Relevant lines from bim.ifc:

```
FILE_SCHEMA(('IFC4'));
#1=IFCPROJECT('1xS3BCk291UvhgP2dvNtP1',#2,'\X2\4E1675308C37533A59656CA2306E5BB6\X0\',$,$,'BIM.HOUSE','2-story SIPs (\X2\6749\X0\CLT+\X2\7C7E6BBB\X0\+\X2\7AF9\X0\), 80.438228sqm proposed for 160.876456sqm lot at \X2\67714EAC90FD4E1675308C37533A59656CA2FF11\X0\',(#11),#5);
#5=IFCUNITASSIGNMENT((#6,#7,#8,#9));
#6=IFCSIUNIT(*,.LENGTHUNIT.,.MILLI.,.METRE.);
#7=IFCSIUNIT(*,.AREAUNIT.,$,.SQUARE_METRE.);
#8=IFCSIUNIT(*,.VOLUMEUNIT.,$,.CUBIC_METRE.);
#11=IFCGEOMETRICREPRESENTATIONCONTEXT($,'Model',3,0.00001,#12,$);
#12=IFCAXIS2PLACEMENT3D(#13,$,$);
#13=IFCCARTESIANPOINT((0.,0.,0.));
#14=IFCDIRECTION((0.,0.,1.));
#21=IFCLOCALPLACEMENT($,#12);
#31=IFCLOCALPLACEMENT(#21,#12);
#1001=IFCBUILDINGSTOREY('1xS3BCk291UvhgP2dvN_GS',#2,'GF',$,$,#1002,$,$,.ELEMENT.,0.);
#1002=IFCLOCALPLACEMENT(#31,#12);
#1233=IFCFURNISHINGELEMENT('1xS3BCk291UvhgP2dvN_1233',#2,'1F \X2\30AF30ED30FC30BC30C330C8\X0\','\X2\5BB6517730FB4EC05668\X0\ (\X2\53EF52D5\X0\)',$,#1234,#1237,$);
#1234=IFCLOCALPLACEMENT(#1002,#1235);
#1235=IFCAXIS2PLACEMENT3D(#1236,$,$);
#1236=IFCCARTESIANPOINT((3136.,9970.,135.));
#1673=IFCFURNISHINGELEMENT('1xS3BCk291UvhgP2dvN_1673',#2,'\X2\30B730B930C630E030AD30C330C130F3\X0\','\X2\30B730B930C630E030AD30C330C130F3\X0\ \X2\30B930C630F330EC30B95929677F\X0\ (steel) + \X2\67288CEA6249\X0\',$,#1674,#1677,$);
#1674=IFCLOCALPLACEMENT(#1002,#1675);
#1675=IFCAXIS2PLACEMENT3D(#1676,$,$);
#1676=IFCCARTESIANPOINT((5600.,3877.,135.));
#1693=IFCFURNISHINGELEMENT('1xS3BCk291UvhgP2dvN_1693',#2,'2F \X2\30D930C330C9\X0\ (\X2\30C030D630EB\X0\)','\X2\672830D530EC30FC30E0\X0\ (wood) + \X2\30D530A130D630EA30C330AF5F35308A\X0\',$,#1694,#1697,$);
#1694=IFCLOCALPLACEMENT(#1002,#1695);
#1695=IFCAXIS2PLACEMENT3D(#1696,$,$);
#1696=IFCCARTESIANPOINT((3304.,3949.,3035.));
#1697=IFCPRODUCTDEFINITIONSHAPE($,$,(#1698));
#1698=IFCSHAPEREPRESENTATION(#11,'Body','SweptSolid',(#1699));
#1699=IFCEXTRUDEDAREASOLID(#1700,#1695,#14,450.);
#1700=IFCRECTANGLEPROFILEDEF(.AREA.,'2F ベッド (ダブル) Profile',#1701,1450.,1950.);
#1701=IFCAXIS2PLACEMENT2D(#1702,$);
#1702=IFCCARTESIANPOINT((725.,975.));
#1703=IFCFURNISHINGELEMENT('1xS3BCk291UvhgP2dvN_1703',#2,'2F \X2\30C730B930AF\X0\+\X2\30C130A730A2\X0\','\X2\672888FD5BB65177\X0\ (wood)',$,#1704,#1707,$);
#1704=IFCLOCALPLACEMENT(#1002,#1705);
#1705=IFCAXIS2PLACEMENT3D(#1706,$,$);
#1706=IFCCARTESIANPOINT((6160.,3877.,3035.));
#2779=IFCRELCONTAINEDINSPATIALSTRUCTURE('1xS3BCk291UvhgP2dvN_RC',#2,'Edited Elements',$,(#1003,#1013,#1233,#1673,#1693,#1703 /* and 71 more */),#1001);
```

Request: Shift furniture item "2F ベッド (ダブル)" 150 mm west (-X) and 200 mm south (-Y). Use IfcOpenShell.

```python
import ifcopenshell
import ifcopenshell.api.geometry
import ifcopenshell.util.placement
import ifcopenshell.util.unit

model = ifcopenshell.open("bim.ifc")
unit_scale = ifcopenshell.util.unit.calculate_unit_scale(model)

item = model.by_guid("1xS3BCk291UvhgP2dvN_1693")
matrix = ifcopenshell.util.placement.get_local_placement(item.ObjectPlacement)
matrix[0, 3] -= 0.15 / unit_scale
matrix[1, 3] -= 0.2 / unit_scale
ifcopenshell.api.geometry.edit_object_placement(model, product=item, matrix=matrix, is_si=False)

print(ifcopenshell.util.placement.get_local_placement(item.ObjectPlacement).round(3) + 0.0)

model.write("bim_updated.ifc")
```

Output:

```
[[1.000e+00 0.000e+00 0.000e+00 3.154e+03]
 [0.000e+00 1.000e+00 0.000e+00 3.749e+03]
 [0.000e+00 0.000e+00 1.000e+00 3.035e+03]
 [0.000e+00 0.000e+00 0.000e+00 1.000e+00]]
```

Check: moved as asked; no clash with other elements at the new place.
